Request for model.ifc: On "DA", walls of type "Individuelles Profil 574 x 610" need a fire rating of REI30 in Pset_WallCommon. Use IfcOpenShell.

First a look at what the model holds.

```python
import ifcopenshell
import ifcopenshell.util.element

model = ifcopenshell.open("model.ifc")
print(model.schema)
storey = next(s for s in model.by_type("IfcBuildingStorey") if s.Name == "DA")
walls = [e for e in ifcopenshell.util.element.get_decomposition(storey) if e.is_a("IfcWall")]
seen = {}
for e in walls:
    element_type = ifcopenshell.util.element.get_type(e)
    key = (element_type.Name if element_type != e and element_type else None, ifcopenshell.util.element.get_pset(e, "Pset_WallCommon", "FireRating"))
    seen[key] = seen.get(key, 0) + 1
for (name, value), count in sorted(seen.items(), key=str):
    print(count, "x", name, "|", value)
```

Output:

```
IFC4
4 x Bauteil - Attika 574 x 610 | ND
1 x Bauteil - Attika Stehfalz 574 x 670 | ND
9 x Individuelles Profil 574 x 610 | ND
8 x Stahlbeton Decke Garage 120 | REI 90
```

```python
import ifcopenshell
import ifcopenshell.api.pset
import ifcopenshell.util.element

model = ifcopenshell.open("model.ifc")

storey = next(s for s in model.by_type("IfcBuildingStorey") if s.Name == "DA")
walls = [e for e in ifcopenshell.util.element.get_decomposition(storey) if e.is_a("IfcWall")]

count = 0
for e in walls:
    element_type = ifcopenshell.util.element.get_type(e)
    if element_type in (None, e) or element_type.Name != "Individuelles Profil 574 x 610":
        continue
    # add_pset returns the element's existing set when there is one.
    pset = ifcopenshell.api.pset.add_pset(model, product=e, name="Pset_WallCommon")
    ifcopenshell.api.pset.edit_pset(model, pset=pset, properties={"FireRating": "REI30"})
    count += 1

print(count, "walls updated")

model.write("model_edited.ifc")
```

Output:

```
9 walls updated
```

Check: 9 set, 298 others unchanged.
